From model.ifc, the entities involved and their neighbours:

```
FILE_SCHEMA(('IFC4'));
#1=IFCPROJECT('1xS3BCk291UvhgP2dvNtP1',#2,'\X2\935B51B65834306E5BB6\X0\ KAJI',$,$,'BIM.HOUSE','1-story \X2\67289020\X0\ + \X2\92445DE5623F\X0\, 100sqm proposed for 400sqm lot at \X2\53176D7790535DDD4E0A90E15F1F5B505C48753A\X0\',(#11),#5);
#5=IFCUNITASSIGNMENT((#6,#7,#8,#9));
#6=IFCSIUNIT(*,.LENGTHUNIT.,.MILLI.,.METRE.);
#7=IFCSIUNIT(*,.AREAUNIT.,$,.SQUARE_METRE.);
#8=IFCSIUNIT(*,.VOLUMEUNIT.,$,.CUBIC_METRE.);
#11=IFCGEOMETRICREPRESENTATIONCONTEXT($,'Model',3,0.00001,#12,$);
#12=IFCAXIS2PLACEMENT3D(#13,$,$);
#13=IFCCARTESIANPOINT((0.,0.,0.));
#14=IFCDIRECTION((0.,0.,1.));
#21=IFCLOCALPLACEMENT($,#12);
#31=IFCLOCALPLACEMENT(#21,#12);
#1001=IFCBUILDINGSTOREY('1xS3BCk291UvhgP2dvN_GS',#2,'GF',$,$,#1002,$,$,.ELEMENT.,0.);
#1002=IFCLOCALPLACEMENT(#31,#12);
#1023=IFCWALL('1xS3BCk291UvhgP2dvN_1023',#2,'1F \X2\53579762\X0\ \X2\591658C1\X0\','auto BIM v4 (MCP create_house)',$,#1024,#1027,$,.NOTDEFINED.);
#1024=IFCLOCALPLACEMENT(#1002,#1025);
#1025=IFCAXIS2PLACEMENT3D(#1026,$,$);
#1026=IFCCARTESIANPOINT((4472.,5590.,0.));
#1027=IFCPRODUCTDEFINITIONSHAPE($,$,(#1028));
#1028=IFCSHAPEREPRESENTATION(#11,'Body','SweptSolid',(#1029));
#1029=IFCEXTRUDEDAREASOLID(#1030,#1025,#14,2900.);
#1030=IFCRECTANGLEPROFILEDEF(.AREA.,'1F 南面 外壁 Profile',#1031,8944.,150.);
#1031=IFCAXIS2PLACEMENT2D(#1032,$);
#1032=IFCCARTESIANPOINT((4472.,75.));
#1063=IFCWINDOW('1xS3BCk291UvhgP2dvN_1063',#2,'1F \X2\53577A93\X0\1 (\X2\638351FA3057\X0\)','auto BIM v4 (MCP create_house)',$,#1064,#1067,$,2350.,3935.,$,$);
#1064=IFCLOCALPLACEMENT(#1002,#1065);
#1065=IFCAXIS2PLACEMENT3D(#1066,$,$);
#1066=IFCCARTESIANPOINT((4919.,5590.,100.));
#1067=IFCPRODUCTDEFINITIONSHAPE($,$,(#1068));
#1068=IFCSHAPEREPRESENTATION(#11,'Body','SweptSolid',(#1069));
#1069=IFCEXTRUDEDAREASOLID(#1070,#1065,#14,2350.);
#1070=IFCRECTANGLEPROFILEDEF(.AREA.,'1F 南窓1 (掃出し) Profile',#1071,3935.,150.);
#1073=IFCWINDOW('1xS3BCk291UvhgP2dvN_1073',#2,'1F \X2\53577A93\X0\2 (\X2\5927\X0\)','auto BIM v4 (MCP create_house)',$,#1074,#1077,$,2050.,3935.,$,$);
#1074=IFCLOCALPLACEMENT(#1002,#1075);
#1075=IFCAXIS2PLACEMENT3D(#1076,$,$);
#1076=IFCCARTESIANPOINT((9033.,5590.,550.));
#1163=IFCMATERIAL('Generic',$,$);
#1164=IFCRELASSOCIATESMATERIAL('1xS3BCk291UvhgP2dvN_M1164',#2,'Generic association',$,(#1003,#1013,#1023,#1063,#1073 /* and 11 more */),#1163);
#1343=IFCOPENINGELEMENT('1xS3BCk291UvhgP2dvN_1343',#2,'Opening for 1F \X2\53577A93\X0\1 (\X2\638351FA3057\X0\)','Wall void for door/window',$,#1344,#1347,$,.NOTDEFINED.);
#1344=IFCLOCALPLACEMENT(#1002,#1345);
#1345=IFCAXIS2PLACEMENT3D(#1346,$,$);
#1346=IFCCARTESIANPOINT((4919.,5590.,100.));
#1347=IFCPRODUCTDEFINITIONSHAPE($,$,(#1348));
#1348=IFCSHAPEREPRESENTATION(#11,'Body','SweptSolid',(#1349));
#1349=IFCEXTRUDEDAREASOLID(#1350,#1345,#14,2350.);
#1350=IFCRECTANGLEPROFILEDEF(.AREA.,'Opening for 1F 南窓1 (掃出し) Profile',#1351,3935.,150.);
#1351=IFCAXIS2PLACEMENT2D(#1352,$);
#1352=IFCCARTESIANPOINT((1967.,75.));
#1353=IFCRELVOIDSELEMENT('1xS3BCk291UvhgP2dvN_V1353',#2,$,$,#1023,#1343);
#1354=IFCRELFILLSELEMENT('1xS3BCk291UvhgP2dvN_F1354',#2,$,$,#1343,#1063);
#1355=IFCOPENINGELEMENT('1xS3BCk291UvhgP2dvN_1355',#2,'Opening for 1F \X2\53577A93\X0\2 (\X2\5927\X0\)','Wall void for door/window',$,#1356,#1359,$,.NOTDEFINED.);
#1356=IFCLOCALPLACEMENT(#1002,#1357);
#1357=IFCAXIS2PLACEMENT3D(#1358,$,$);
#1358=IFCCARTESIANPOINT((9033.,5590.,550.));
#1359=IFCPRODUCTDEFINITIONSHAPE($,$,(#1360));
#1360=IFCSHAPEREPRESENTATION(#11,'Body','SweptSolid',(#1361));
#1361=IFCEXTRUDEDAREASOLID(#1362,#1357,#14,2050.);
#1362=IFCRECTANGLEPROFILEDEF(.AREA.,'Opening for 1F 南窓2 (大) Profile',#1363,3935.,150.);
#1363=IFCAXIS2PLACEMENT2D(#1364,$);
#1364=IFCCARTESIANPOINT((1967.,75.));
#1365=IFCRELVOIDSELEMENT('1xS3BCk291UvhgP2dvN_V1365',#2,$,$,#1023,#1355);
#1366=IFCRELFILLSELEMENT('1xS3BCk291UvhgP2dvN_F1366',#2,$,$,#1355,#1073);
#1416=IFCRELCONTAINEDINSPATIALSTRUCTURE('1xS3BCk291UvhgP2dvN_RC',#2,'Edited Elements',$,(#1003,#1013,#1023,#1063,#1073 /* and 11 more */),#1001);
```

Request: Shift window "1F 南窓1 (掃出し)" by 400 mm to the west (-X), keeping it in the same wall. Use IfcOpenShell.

```python
import ifcopenshell
import ifcopenshell.api.geometry
import ifcopenshell.util.placement

model = ifcopenshell.open("model.ifc")

window = model.by_guid("1xS3BCk291UvhgP2dvN_1063")
opening = window.FillsVoids[0].RelatingOpeningElement
wall = opening.VoidsElements[0].RelatingBuildingElement

wall_matrix = ifcopenshell.util.placement.get_local_placement(wall.ObjectPlacement)
shift = wall_matrix[:3, 0] * -400.0
before = ifcopenshell.util.placement.get_local_placement(window.ObjectPlacement)[:3, 3].copy()

# The window is not placed relative to its opening, so move both.
for product in (opening, window):
    matrix = ifcopenshell.util.placement.get_local_placement(product.ObjectPlacement)
    matrix[:3, 3] += shift
    ifcopenshell.api.geometry.edit_object_placement(model, product=product, matrix=matrix, is_si=False)

after = ifcopenshell.util.placement.get_local_placement(window.ObjectPlacement)[:3, 3]
print("window moved by", (after - before).round(3) + 0.0)

model.write("model_edited.ifc")
```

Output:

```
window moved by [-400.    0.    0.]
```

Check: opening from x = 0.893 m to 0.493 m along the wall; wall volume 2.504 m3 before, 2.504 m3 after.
